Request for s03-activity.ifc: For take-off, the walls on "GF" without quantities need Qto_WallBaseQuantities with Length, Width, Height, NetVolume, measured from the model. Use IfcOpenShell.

First a look at what the model holds.

```python
import ifcopenshell
import ifcopenshell.util.element
import ifcopenshell.util.unit

model = ifcopenshell.open("s03-activity.ifc")
print(model.schema)
for unit_type in ("LENGTHUNIT", "AREAUNIT", "VOLUMEUNIT"):
    print(unit_type, ifcopenshell.util.unit.calculate_unit_scale(model, unit_type))
storey = next(s for s in model.by_type("IfcBuildingStorey") if s.Name == "GF")
walls = [e for e in ifcopenshell.util.element.get_decomposition(storey) if e.is_a("IfcWall")]
for e in sorted(walls, key=lambda e: e.id()):
    print(e.id(), e.is_a(), e.Name, list(ifcopenshell.util.element.get_psets(e, qtos_only=True)), sep=" | ")
```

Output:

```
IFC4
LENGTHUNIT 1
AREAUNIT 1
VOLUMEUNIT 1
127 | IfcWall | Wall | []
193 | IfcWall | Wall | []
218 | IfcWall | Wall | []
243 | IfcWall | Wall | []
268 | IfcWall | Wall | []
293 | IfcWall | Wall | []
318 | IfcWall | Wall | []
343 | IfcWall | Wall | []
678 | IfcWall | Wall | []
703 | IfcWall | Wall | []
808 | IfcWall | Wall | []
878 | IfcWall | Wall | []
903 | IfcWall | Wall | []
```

```python
import ifcopenshell
import ifcopenshell.api.pset
import ifcopenshell.geom
import ifcopenshell.util.element
import ifcopenshell.util.shape
import ifcopenshell.util.unit

model = ifcopenshell.open("s03-activity.ifc")
unit_scale = ifcopenshell.util.unit.calculate_unit_scale(model)
volume_scale = ifcopenshell.util.unit.calculate_unit_scale(model, "VOLUMEUNIT")
settings = ifcopenshell.geom.settings()

storey = next(s for s in model.by_type("IfcBuildingStorey") if s.Name == "GF")
walls = [e for e in ifcopenshell.util.element.get_decomposition(storey) if e.is_a("IfcWall")]

for e in sorted(walls, key=lambda e: e.id()):
    if ifcopenshell.util.element.get_psets(e, qtos_only=True, should_inherit=False):
        continue
    # Geometry comes back in metres, in the element's own axes.
    shape = ifcopenshell.geom.create_shape(settings, e)
    values = {
        "Length": ifcopenshell.util.shape.get_x(shape.geometry) / unit_scale,
        "Width": ifcopenshell.util.shape.get_y(shape.geometry) / unit_scale,
        "Height": ifcopenshell.util.shape.get_z(shape.geometry) / unit_scale,
        "NetVolume": ifcopenshell.util.shape.get_volume(shape.geometry) / volume_scale,
    }
    qto = ifcopenshell.api.pset.add_qto(model, product=e, name="Qto_WallBaseQuantities")
    ifcopenshell.api.pset.edit_qto(model, qto=qto, properties=values)
    print(e.id(), {k: round(v, 3) for k, v in values.items()})

model.write("s03-activity_updated.ifc")
```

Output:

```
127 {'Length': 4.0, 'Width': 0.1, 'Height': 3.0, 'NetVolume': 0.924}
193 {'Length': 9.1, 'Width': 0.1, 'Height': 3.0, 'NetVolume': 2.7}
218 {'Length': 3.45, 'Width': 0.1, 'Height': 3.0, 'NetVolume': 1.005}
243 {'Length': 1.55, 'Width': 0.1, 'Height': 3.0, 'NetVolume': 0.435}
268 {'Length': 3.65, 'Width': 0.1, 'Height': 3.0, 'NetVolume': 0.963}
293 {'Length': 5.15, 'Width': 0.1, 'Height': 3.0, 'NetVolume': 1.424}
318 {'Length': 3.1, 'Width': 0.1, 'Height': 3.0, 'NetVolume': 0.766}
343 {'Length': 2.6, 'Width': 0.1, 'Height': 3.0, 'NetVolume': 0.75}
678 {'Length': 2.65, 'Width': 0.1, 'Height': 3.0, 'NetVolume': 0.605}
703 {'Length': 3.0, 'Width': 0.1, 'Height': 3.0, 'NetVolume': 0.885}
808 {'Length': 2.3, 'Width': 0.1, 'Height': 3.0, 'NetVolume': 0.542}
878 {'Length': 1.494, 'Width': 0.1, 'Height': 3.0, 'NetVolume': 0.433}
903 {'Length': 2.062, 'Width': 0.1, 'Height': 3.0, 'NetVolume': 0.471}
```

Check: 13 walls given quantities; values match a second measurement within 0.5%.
